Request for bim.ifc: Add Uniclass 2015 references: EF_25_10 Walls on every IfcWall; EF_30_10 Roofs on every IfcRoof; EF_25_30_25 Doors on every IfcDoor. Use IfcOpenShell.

First a look at what the model holds.

```python
import ifcopenshell

model = ifcopenshell.open("bim.ifc")
print(model.schema)
print("classifications:", [c.Name for c in model.by_type("IfcClassification")])
for ifc_class in ("IfcDoor", "IfcRoof", "IfcStair", "IfcWall", "IfcWindow"):
    print(ifc_class, len(model.by_type(ifc_class)))
```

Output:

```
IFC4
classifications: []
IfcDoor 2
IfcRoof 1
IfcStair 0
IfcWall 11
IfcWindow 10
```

```python
import ifcopenshell
import ifcopenshell.api.classification

model = ifcopenshell.open("bim.ifc")

system = ifcopenshell.api.classification.add_classification(model, classification="Uniclass 2015")

codes = {
    "IfcWall": ("EF_25_10", "Walls"),
    "IfcRoof": ("EF_30_10", "Roofs"),
    "IfcDoor": ("EF_25_30_25", "Doors"),
}
for ifc_class, (code, name) in codes.items():
    products = model.by_type(ifc_class)
    ifcopenshell.api.classification.add_reference(
        model, products=products, classification=system, identification=code, name=name
    )
    print(code, len(products))

model.write("bim_v2.ifc")
```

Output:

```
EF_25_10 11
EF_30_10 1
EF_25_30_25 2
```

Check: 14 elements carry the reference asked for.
